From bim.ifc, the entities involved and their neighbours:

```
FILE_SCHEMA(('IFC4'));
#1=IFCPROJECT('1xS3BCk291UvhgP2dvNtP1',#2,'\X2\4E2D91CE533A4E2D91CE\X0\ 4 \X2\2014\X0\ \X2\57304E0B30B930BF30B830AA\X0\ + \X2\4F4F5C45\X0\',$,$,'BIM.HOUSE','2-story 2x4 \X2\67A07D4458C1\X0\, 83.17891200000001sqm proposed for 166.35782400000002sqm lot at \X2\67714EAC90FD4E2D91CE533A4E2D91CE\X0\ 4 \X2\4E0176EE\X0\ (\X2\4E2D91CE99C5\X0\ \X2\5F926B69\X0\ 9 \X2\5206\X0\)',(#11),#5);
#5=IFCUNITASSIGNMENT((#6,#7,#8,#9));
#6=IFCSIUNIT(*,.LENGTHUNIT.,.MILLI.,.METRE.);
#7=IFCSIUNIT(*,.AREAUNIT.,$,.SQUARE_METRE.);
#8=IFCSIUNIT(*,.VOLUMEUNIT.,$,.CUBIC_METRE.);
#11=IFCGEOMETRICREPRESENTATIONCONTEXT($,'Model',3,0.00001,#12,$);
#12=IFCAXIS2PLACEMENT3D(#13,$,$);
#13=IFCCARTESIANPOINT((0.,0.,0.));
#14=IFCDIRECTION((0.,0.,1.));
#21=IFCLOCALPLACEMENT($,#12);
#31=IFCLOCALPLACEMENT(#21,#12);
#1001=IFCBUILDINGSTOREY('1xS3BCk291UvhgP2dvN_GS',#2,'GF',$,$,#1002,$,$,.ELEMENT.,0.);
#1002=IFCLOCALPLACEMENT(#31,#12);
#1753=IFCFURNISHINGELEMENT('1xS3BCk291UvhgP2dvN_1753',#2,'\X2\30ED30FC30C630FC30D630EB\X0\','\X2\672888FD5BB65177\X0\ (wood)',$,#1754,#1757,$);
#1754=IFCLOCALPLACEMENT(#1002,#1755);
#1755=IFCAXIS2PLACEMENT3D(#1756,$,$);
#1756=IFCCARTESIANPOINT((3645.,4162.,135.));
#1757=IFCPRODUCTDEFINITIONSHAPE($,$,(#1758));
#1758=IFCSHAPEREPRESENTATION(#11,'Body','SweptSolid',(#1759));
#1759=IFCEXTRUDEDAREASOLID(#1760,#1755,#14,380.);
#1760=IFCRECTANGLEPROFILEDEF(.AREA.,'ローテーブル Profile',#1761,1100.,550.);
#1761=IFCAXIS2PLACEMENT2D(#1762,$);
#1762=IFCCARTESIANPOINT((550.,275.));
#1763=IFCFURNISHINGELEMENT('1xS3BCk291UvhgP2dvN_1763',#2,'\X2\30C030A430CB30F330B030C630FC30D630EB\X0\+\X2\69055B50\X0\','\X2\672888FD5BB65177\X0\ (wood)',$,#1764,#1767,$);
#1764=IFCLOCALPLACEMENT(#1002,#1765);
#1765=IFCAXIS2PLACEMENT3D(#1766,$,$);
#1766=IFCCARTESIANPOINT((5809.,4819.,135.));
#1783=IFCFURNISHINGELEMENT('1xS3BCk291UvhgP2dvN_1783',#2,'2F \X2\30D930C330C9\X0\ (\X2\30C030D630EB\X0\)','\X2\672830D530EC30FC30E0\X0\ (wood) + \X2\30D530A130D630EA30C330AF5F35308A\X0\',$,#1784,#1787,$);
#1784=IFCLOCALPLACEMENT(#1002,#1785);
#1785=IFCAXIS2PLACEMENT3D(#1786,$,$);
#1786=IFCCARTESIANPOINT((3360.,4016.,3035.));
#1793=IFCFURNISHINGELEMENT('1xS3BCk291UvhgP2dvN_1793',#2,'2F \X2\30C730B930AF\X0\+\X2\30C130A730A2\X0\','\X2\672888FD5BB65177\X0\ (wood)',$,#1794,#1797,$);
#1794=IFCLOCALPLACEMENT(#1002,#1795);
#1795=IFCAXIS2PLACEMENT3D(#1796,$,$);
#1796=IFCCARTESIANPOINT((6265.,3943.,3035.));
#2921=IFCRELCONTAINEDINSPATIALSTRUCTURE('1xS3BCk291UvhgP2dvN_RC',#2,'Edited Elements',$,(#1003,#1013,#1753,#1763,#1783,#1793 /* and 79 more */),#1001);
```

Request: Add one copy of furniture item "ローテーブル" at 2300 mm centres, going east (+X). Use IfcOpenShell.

```python
import numpy as np
import ifcopenshell
import ifcopenshell.api.geometry
import ifcopenshell.api.root
import ifcopenshell.util.element
import ifcopenshell.util.placement

model = ifcopenshell.open("bim.ifc")


def reuse_history(source, copy):
    """copy_class also copies each property set's owner history, people and application; keep the originals."""
    for rel in copy.IsDefinedBy:
        if rel.is_a("IfcRelDefinesByProperties") and (history := rel.RelatingPropertyDefinition.OwnerHistory):
            rel.RelatingPropertyDefinition.OwnerHistory = source.OwnerHistory
            ifcopenshell.util.element.remove_deep2(model, history)


source = model.by_guid("1xS3BCk291UvhgP2dvN_1753")
base = ifcopenshell.util.placement.get_local_placement(source.ObjectPlacement)
step = np.array([1.0, 0.0, 0.0]) * 2300.0

for i in range(1, 2):
    copy = ifcopenshell.api.root.copy_class(model, product=source)
    copy.Representation = ifcopenshell.util.element.copy_deep(
        model, source.Representation, exclude=["IfcGeometricRepresentationContext", "IfcRepresentationMap"]
    )
    reuse_history(source, copy)
    matrix = base.copy()
    matrix[:3, 3] += i * step
    print("added at", matrix[:3, 3].round(3) + 0.0)
    ifcopenshell.api.geometry.edit_object_placement(model, product=copy, matrix=matrix, is_si=False)

model.write("bim_v2.ifc")
```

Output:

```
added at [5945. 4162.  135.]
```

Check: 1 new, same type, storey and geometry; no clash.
